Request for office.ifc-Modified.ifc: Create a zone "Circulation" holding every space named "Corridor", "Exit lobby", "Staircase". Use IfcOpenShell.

First a look at what the model holds.

```python
import ifcopenshell

model = ifcopenshell.open("office.ifc-Modified.ifc")
print(model.schema)
seen = {}
for space in model.by_type("IfcSpace"):
    seen[space.LongName] = seen.get(space.LongName, 0) + 1
for name, count in sorted(seen.items(), key=str):
    print(count, "x", name)
print("zones:", [z.Name for z in model.by_type("IfcZone")][:20])
```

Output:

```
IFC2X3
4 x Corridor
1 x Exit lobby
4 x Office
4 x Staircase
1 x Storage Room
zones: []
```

```python
import ifcopenshell
import ifcopenshell.api.group
import ifcopenshell.api.root

model = ifcopenshell.open("office.ifc-Modified.ifc")

names = {"Corridor", "Exit lobby", "Staircase"}
spaces = [s for s in model.by_type("IfcSpace") if s.LongName in names]

zone = ifcopenshell.api.root.create_entity(model, ifc_class="IfcZone", name="Circulation")
ifcopenshell.api.group.assign_group(model, products=spaces, group=zone)
print(len(spaces), "spaces in", zone.Name)

model.write("office.ifc-Modified_rev.ifc")
```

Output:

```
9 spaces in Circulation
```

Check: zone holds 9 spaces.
